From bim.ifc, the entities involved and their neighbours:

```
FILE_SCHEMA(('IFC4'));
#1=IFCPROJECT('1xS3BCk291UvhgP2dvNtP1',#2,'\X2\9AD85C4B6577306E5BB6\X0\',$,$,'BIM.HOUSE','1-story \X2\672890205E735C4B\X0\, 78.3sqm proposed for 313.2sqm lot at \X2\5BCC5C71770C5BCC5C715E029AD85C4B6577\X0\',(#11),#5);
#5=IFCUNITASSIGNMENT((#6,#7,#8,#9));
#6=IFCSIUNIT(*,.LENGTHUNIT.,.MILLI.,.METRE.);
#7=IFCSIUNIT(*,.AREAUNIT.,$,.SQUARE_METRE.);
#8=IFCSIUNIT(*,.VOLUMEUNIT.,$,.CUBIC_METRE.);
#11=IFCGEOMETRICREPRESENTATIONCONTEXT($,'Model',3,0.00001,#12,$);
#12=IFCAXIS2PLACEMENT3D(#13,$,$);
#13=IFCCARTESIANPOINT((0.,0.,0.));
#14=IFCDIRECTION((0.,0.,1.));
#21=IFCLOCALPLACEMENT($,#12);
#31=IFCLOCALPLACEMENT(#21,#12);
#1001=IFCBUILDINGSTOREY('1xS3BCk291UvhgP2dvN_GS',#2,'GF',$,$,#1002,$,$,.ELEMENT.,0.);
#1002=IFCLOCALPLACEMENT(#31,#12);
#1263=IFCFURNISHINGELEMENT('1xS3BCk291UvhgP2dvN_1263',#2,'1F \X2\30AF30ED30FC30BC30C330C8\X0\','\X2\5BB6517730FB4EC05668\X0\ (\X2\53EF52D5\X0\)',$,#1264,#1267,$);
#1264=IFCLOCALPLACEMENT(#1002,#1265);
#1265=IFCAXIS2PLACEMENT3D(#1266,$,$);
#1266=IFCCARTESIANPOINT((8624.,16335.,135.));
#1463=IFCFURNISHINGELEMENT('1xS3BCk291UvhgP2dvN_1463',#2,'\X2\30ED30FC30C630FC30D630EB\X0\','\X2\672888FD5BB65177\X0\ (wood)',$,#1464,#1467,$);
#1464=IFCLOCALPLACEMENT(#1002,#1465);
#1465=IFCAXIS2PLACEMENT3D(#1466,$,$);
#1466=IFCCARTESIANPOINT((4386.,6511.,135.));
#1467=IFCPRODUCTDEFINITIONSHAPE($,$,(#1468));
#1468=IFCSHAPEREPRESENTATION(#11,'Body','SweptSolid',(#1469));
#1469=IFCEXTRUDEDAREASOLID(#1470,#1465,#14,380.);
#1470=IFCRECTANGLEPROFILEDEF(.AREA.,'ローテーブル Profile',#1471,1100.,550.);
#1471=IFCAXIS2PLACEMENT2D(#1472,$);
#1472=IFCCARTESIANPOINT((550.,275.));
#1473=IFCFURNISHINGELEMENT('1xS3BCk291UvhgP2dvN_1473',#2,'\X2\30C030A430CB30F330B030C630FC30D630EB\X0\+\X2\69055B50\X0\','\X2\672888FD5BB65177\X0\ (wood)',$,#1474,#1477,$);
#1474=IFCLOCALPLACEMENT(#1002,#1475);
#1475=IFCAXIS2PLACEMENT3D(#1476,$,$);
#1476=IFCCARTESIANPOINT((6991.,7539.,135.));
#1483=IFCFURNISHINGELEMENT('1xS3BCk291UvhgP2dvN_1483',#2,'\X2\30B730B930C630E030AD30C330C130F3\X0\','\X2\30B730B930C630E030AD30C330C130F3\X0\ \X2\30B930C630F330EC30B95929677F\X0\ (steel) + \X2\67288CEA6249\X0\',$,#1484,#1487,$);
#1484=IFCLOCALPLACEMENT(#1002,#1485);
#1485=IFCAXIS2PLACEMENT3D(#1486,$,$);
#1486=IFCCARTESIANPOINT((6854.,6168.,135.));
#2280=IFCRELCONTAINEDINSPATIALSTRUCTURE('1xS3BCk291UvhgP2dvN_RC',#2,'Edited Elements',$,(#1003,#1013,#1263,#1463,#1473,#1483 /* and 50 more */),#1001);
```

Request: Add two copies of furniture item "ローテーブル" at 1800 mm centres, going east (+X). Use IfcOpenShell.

```python
import numpy as np
import ifcopenshell
import ifcopenshell.api.geometry
import ifcopenshell.api.root
import ifcopenshell.util.element
import ifcopenshell.util.placement
import ifcopenshell.util.unit

model = ifcopenshell.open("bim.ifc")
unit_scale = ifcopenshell.util.unit.calculate_unit_scale(model)


def reuse_history(source, copy):
    """copy_class also copies each property set's owner history, people and application; keep the originals."""
    for rel in copy.IsDefinedBy:
        if rel.is_a("IfcRelDefinesByProperties") and (history := rel.RelatingPropertyDefinition.OwnerHistory):
            rel.RelatingPropertyDefinition.OwnerHistory = source.OwnerHistory
            ifcopenshell.util.element.remove_deep2(model, history)


source = model.by_guid("1xS3BCk291UvhgP2dvN_1463")
base = ifcopenshell.util.placement.get_local_placement(source.ObjectPlacement)
step = np.array([1.0, 0.0, 0.0]) * 1.8 / unit_scale

for i in range(1, 3):
    copy = ifcopenshell.api.root.copy_class(model, product=source)
    copy.Representation = ifcopenshell.util.element.copy_deep(
        model, source.Representation, exclude=["IfcGeometricRepresentationContext", "IfcRepresentationMap"]
    )
    reuse_history(source, copy)
    matrix = base.copy()
    matrix[:3, 3] += i * step
    print("added at", matrix[:3, 3].round(3) + 0.0)
    ifcopenshell.api.geometry.edit_object_placement(model, product=copy, matrix=matrix, is_si=False)

model.write("bim_updated.ifc")
```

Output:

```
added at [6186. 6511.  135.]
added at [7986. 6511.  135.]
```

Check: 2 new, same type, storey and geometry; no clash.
